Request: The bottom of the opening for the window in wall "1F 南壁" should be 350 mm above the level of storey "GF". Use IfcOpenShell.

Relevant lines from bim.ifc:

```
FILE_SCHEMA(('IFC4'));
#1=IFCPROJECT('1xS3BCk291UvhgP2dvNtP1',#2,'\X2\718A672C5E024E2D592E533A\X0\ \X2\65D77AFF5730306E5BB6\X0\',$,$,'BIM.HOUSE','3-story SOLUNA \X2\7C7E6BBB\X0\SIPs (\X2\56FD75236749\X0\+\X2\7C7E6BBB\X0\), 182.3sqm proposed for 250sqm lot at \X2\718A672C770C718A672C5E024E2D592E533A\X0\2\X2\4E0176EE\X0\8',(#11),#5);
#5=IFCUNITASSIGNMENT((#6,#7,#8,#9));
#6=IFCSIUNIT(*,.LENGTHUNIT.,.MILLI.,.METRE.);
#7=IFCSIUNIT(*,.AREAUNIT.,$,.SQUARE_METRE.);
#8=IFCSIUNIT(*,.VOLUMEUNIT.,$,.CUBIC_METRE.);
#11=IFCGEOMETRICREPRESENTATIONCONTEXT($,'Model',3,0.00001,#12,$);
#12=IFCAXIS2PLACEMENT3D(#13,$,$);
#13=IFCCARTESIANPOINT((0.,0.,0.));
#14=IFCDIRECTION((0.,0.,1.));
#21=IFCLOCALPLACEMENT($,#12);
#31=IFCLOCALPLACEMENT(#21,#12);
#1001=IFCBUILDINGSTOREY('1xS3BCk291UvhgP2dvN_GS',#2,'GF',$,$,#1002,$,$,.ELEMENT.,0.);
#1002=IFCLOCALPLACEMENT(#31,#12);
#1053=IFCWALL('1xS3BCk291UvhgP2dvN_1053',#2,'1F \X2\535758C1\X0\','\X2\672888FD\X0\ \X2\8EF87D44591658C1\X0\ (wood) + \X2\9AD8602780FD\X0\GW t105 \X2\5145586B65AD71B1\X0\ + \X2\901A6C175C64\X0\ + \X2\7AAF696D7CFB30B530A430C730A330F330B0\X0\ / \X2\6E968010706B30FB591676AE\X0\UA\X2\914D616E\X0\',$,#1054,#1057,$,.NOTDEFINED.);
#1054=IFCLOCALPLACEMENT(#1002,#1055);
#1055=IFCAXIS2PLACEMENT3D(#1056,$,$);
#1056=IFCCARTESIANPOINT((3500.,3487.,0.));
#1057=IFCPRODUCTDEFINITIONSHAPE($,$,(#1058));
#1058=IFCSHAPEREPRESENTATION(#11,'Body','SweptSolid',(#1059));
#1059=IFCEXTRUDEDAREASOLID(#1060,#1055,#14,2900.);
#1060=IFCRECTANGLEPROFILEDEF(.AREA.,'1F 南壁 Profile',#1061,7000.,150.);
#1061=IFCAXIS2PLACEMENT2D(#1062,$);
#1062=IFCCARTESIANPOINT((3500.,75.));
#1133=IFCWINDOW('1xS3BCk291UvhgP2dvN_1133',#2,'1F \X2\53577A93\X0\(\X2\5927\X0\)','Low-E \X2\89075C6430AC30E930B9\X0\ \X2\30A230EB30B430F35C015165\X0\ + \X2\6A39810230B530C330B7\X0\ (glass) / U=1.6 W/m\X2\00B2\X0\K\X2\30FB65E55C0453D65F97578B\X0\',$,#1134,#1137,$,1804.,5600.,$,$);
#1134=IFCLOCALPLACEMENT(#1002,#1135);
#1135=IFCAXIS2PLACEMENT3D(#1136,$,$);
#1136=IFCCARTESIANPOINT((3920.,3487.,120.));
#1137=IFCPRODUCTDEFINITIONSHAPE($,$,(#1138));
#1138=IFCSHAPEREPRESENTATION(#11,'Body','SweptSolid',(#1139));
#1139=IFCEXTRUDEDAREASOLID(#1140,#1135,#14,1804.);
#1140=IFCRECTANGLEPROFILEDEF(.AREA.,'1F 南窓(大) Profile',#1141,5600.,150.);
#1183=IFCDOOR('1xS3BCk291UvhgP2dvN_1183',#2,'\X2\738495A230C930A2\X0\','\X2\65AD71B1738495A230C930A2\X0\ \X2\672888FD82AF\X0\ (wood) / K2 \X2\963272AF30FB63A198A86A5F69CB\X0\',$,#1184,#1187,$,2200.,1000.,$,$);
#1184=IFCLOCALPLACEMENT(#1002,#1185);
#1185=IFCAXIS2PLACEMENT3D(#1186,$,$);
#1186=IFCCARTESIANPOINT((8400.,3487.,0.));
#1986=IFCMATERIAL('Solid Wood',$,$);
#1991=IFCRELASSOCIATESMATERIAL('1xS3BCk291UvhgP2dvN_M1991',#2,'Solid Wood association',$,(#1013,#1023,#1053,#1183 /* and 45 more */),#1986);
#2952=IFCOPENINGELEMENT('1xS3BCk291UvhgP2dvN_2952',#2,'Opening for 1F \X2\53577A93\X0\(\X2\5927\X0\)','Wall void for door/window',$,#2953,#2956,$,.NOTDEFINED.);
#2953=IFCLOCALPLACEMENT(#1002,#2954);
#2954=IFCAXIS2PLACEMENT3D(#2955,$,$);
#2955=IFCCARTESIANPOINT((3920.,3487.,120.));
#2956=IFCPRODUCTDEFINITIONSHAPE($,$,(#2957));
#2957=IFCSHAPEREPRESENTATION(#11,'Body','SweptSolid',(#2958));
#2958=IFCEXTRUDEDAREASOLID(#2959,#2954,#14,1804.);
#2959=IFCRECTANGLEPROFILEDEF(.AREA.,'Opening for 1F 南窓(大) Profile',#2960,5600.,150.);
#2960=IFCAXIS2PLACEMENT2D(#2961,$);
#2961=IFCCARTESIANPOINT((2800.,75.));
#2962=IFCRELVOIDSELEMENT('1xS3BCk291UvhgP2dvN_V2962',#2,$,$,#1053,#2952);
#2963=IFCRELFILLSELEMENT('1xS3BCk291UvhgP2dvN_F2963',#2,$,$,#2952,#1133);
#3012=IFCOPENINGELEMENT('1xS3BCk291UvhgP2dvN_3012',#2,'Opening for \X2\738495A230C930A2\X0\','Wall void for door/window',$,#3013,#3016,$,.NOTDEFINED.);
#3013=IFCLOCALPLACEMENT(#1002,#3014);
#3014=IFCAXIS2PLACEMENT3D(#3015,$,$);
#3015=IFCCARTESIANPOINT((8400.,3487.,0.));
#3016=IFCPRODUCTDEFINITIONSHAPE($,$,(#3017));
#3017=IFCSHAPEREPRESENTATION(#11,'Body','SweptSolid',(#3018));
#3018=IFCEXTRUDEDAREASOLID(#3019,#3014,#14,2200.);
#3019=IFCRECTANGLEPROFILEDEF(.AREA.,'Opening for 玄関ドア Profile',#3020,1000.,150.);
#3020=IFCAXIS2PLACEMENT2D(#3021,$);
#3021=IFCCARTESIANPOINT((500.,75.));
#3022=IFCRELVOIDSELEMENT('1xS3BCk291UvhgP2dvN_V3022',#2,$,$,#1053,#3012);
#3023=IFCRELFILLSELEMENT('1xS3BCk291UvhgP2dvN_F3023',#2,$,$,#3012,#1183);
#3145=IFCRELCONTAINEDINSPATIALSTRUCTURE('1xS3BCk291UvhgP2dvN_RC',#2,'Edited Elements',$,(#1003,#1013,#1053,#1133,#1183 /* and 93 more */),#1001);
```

```python
import numpy as np
import ifcopenshell
import ifcopenshell.api.geometry
import ifcopenshell.geom
import ifcopenshell.util.element
import ifcopenshell.util.placement
import ifcopenshell.util.shape
import ifcopenshell.util.unit

model = ifcopenshell.open("bim.ifc")
unit_scale = ifcopenshell.util.unit.calculate_unit_scale(model)

window = model.by_guid("1xS3BCk291UvhgP2dvN_1133")
opening = window.FillsVoids[0].RelatingOpeningElement
storey = ifcopenshell.util.element.get_container(window, ifc_class="IfcBuildingStorey")
level = ifcopenshell.util.placement.get_local_placement(storey.ObjectPlacement)[2, 3]

# The opening's origin need not be at the sill, so measure its lowest point.
shape = ifcopenshell.geom.create_shape(ifcopenshell.geom.settings(), opening)
bottom = ifcopenshell.util.shape.get_shape_bottom_elevation(shape, shape.geometry) / unit_scale
dz = level + 0.35 / unit_scale - bottom

shift = np.array([0.0, 0.0, dz])
# The window is not placed relative to its opening, so move both.
for product in (opening, window):
    matrix = ifcopenshell.util.placement.get_local_placement(product.ObjectPlacement)
    matrix[:3, 3] += shift
    ifcopenshell.api.geometry.edit_object_placement(model, product=product, matrix=matrix, is_si=False)

print(f"moved by {dz * unit_scale:+.3f} m")

model.write("bim-out.ifc")
```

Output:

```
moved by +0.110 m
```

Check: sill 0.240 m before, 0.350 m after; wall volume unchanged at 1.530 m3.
